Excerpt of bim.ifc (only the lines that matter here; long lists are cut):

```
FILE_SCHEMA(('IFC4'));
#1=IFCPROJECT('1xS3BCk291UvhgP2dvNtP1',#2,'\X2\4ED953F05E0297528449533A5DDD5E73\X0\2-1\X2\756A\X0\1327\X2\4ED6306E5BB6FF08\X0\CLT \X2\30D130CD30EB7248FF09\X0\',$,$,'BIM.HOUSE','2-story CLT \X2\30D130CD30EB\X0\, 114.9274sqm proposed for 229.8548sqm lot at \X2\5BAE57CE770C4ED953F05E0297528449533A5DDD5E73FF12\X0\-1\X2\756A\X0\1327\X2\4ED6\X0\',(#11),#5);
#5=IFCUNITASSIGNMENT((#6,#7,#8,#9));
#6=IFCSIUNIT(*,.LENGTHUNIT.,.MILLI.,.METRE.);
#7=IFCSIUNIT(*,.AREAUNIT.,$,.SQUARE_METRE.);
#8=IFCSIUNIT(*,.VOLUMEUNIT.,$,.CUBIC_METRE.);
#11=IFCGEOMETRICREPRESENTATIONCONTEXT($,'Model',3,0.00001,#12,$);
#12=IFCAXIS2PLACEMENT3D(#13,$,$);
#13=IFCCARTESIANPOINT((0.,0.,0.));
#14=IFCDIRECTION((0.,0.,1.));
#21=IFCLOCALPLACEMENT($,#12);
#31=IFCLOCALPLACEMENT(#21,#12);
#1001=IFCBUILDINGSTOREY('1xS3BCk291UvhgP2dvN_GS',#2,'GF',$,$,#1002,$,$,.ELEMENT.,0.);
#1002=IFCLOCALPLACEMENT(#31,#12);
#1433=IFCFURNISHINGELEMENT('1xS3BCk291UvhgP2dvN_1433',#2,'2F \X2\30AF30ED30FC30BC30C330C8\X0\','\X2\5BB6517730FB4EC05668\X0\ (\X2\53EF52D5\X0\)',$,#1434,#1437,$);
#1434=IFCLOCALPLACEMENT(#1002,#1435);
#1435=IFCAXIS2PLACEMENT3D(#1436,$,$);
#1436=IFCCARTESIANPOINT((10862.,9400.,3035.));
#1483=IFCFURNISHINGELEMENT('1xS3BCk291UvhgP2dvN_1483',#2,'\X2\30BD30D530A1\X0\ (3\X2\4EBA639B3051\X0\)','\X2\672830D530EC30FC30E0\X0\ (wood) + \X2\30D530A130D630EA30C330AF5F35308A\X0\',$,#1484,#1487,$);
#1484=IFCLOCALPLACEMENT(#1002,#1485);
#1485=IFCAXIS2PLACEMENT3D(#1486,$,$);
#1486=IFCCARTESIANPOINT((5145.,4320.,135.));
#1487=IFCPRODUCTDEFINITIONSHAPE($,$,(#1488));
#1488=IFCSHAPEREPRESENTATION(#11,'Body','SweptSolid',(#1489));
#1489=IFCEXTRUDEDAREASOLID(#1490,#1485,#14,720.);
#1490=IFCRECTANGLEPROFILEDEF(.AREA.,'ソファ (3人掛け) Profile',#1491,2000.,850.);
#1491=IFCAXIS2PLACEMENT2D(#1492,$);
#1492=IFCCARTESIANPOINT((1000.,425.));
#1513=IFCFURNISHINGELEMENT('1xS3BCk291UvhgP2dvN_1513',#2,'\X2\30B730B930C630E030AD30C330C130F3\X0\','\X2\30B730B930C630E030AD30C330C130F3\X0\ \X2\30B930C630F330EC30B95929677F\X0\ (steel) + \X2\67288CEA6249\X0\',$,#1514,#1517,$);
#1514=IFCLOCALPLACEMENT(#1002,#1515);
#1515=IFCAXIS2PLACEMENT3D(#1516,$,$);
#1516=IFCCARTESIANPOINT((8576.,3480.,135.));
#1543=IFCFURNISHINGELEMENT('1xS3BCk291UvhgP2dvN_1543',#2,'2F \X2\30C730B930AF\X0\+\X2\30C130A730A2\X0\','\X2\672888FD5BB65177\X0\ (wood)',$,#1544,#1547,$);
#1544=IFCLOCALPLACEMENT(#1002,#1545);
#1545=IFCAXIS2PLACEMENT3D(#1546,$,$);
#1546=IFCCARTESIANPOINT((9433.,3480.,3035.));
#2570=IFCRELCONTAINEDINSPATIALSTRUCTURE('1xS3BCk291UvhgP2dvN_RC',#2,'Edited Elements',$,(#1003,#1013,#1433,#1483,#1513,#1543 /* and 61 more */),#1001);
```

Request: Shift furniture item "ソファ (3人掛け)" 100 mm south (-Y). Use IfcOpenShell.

```python
import ifcopenshell
import ifcopenshell.api.geometry
import ifcopenshell.util.placement

model = ifcopenshell.open("bim.ifc")

item = model.by_id(1483)
matrix = ifcopenshell.util.placement.get_local_placement(item.ObjectPlacement)
matrix[1, 3] -= 100.0
ifcopenshell.api.geometry.edit_object_placement(model, product=item, matrix=matrix, is_si=False)

print(ifcopenshell.util.placement.get_local_placement(item.ObjectPlacement).round(3) + 0.0)

model.write("bim_v2.ifc")
```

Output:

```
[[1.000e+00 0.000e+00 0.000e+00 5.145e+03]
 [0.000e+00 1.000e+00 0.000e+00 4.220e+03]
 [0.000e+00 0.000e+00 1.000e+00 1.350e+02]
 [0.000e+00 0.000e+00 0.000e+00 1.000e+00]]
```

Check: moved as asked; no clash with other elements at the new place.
